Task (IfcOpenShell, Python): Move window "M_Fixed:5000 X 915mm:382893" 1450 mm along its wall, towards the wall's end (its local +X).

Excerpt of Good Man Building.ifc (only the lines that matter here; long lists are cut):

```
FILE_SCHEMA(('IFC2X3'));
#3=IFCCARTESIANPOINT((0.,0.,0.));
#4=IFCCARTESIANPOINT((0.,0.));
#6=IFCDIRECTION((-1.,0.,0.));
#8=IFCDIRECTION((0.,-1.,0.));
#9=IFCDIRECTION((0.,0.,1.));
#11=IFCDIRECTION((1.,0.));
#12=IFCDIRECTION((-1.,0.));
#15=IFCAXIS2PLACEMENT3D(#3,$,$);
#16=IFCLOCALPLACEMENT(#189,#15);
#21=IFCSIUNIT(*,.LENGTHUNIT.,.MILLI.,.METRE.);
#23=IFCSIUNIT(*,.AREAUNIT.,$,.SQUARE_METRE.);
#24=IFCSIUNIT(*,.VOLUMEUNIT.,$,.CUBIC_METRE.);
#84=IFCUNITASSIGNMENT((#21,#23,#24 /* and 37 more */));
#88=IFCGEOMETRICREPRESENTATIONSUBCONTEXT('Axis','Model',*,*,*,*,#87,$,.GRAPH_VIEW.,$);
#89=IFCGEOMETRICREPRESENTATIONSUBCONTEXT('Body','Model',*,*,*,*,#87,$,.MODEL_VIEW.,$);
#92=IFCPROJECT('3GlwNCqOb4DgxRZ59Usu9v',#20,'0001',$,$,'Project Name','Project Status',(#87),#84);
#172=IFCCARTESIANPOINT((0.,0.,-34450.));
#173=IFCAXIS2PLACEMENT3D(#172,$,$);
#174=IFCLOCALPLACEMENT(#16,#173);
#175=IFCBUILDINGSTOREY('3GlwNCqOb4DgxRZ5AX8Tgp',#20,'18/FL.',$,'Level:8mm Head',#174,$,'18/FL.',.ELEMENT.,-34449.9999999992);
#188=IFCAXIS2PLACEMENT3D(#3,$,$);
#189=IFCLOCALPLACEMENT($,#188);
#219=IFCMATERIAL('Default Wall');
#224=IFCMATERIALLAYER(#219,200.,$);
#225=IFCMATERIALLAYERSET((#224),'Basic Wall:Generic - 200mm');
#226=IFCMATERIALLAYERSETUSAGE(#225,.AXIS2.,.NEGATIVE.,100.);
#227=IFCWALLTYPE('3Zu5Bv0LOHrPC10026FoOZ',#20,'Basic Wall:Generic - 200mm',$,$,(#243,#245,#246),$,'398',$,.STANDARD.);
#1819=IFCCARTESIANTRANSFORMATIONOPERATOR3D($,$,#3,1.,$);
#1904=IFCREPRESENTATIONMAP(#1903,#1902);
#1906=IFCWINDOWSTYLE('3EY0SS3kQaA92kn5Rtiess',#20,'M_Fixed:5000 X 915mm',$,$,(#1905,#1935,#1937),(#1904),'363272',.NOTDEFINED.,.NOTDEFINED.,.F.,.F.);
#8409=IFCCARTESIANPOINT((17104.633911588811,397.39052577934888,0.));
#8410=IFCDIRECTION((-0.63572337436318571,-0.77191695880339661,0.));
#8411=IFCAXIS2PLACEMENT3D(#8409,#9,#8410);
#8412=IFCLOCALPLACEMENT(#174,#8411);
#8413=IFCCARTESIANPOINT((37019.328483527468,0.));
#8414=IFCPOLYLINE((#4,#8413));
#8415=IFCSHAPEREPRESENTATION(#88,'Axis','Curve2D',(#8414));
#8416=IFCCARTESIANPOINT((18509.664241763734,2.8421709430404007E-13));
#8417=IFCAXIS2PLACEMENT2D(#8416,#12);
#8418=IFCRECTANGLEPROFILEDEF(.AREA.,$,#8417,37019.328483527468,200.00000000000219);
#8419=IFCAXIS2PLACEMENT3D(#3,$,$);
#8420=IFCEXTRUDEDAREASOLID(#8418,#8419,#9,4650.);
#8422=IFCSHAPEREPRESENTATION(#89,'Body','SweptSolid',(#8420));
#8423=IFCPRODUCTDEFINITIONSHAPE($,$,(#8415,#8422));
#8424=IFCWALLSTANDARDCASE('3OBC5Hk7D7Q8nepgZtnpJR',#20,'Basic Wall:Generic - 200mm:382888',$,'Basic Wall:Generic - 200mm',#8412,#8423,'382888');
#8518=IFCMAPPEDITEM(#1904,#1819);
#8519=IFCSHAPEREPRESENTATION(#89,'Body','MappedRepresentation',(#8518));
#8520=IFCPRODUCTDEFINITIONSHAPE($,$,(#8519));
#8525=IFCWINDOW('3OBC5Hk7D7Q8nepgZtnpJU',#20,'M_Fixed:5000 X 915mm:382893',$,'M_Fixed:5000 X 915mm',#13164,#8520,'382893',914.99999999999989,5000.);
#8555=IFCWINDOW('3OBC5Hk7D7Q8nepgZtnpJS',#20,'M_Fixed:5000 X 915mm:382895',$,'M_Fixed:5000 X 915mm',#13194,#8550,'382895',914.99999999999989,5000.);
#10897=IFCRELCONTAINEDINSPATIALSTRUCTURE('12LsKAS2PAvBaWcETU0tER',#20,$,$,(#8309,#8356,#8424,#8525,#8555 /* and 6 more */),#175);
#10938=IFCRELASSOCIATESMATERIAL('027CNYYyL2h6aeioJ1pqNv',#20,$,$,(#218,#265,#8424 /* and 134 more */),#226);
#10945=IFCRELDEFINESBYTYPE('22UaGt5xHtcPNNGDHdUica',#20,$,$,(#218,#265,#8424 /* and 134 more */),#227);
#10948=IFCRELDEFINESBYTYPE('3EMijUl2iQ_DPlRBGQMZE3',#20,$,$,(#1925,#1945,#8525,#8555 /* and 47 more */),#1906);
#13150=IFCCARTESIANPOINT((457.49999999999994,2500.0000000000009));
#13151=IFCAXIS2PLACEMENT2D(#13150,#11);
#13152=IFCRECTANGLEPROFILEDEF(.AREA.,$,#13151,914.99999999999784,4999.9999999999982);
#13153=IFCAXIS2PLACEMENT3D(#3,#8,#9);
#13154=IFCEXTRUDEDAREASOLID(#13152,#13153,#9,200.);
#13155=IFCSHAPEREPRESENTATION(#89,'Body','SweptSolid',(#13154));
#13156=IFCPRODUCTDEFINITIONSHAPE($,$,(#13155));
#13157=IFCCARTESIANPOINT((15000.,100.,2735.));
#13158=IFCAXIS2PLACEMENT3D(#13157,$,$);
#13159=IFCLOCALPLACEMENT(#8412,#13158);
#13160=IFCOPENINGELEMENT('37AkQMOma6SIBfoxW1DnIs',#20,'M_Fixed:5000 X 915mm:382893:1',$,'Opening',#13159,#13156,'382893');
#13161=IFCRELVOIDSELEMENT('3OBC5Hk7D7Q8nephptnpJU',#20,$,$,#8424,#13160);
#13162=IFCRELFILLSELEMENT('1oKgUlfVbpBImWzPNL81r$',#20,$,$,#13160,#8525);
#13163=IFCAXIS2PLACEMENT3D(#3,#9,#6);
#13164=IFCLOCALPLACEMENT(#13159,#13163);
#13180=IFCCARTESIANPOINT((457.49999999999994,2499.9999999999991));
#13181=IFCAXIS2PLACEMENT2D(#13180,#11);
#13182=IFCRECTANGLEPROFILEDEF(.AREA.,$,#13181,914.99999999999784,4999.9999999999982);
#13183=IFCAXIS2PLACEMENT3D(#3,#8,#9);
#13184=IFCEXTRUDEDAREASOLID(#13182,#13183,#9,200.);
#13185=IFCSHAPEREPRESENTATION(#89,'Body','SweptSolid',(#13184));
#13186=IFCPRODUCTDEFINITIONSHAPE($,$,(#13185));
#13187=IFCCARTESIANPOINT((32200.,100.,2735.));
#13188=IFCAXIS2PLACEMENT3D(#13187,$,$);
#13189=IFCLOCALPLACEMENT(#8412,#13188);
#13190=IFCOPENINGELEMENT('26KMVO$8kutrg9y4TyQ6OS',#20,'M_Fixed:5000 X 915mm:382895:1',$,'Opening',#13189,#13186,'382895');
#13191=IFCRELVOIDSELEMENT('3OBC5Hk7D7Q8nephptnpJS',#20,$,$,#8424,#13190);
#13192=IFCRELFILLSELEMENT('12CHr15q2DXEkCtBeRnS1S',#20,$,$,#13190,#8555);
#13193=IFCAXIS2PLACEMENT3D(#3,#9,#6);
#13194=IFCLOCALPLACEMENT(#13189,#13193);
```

```python
import ifcopenshell
import ifcopenshell.api.geometry
import ifcopenshell.util.placement

model = ifcopenshell.open("Good Man Building.ifc")

window = model.by_guid("3OBC5Hk7D7Q8nepgZtnpJU")
opening = window.FillsVoids[0].RelatingOpeningElement
wall = opening.VoidsElements[0].RelatingBuildingElement

wall_matrix = ifcopenshell.util.placement.get_local_placement(wall.ObjectPlacement)
shift = wall_matrix[:3, 0] * 1450.0
before = ifcopenshell.util.placement.get_local_placement(window.ObjectPlacement)[:3, 3].copy()

# The window is placed relative to its opening, so it follows when the opening moves.
matrix = ifcopenshell.util.placement.get_local_placement(opening.ObjectPlacement)
matrix[:3, 3] += shift
ifcopenshell.api.geometry.edit_object_placement(
    model, product=opening, matrix=matrix, is_si=False, should_transform_children=True
)

after = ifcopenshell.util.placement.get_local_placement(window.ObjectPlacement)[:3, 3]
print("window moved by", (after - before).round(3) + 0.0)

model.write("Good Man Building_rev.ifc")
```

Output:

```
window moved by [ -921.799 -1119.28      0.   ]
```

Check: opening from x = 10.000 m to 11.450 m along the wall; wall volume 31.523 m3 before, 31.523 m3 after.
